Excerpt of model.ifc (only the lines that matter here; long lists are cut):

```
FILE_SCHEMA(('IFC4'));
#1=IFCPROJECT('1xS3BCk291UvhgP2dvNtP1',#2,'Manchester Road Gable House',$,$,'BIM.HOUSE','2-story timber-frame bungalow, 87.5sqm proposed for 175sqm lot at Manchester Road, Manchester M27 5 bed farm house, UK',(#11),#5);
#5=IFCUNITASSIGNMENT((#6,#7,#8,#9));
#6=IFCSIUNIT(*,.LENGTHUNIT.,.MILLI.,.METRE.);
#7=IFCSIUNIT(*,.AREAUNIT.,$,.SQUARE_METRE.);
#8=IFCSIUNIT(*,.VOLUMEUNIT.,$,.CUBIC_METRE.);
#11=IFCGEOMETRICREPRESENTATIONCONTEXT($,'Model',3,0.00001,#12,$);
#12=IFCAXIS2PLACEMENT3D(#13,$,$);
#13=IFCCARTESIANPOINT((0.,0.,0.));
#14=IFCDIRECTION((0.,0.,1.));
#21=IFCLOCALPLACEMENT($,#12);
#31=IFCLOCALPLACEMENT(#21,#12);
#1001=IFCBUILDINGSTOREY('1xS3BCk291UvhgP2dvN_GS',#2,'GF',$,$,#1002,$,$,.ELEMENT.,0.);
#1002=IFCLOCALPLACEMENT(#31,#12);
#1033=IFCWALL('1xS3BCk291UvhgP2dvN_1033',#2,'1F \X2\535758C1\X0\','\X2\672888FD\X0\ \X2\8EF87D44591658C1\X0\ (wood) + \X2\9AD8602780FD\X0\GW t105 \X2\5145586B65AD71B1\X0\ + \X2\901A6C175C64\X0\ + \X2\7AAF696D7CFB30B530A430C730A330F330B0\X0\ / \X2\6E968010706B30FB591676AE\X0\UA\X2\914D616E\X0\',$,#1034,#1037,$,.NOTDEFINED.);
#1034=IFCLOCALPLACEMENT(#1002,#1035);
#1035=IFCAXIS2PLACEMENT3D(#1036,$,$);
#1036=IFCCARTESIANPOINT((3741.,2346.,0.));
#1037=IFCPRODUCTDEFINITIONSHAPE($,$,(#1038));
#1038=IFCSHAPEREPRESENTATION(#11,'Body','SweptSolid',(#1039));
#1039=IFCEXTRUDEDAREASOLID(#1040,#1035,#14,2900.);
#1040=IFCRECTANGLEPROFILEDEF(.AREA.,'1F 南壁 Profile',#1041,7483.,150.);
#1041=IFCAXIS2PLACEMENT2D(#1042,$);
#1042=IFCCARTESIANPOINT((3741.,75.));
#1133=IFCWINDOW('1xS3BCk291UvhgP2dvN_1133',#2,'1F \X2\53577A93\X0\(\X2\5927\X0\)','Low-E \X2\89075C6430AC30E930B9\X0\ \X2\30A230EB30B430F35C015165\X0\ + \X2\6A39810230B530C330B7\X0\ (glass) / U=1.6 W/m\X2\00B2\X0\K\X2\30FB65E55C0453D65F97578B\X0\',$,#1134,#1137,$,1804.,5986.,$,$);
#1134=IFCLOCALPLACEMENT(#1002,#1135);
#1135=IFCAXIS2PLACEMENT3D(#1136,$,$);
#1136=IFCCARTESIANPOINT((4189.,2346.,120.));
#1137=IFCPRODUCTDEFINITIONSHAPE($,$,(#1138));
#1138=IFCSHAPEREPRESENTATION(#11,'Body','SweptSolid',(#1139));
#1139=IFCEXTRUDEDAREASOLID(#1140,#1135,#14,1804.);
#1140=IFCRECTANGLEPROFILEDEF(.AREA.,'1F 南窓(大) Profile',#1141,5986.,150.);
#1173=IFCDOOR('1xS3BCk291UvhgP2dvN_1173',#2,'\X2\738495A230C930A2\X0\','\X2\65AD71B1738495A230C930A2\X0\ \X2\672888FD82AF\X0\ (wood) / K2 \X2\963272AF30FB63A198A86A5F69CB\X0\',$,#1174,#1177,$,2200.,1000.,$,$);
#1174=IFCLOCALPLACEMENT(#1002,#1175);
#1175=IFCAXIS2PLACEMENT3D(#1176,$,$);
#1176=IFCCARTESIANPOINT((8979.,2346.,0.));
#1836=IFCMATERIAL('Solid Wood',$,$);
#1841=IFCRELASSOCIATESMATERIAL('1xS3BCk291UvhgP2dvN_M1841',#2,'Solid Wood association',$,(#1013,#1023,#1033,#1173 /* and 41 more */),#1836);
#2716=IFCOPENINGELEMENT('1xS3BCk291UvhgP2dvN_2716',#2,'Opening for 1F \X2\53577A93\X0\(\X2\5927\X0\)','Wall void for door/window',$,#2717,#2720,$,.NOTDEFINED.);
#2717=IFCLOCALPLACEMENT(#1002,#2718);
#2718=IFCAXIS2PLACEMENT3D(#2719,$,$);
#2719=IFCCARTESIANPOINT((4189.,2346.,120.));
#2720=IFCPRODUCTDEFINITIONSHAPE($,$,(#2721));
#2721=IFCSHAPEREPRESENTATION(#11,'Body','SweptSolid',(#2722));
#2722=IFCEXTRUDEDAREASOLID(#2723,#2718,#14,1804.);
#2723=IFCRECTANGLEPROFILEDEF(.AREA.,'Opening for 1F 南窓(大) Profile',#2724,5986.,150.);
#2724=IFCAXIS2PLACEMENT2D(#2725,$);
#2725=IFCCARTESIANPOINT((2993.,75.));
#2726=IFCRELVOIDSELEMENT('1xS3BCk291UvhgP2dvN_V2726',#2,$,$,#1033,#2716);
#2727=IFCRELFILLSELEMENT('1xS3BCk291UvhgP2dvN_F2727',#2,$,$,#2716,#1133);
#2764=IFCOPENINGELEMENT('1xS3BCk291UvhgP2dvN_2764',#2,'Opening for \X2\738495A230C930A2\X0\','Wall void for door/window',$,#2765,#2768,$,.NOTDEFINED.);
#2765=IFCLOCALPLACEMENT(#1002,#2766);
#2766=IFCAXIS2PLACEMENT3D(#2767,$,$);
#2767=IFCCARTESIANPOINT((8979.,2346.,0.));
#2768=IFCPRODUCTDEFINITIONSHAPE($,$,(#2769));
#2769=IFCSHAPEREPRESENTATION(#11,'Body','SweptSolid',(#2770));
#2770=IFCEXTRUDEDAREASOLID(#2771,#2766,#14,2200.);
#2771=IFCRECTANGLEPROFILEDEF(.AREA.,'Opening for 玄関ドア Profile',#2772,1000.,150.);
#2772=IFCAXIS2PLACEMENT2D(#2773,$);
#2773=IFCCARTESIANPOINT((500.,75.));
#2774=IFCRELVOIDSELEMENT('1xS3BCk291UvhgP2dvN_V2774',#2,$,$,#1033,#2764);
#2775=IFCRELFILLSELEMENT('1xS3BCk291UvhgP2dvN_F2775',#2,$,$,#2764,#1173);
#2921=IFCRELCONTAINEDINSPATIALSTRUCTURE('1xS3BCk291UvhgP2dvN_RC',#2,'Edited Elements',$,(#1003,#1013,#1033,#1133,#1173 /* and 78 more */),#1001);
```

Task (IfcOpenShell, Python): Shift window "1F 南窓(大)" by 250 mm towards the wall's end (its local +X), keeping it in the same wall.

```python
import ifcopenshell
import ifcopenshell.api.geometry
import ifcopenshell.util.placement
import ifcopenshell.util.unit

model = ifcopenshell.open("model.ifc")
unit_scale = ifcopenshell.util.unit.calculate_unit_scale(model)

window = model.by_guid("1xS3BCk291UvhgP2dvN_1133")
opening = window.FillsVoids[0].RelatingOpeningElement
wall = opening.VoidsElements[0].RelatingBuildingElement

wall_matrix = ifcopenshell.util.placement.get_local_placement(wall.ObjectPlacement)
shift = wall_matrix[:3, 0] * 0.25 / unit_scale
before = ifcopenshell.util.placement.get_local_placement(window.ObjectPlacement)[:3, 3].copy()

# The window is not placed relative to its opening, so move both.
for product in (opening, window):
    matrix = ifcopenshell.util.placement.get_local_placement(product.ObjectPlacement)
    matrix[:3, 3] += shift
    ifcopenshell.api.geometry.edit_object_placement(model, product=product, matrix=matrix, is_si=False)

after = ifcopenshell.util.placement.get_local_placement(window.ObjectPlacement)[:3, 3]
print("window moved by", (after - before).round(3) + 0.0)

model.write("model_rev.ifc")
```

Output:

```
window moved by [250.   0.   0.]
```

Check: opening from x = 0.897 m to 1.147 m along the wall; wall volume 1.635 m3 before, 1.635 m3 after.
